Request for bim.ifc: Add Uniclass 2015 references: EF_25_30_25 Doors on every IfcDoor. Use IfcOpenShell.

First a look at what the model holds.

```python
import ifcopenshell

model = ifcopenshell.open("bim.ifc")
print(model.schema)
print("classifications:", [c.Name for c in model.by_type("IfcClassification")])
for ifc_class in ("IfcDoor", "IfcRoof", "IfcStair", "IfcWall", "IfcWindow"):
    print(ifc_class, len(model.by_type(ifc_class)))
```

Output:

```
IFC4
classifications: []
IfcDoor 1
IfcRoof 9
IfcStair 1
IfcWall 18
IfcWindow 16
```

```python
import ifcopenshell
import ifcopenshell.api.classification

model = ifcopenshell.open("bim.ifc")

system = ifcopenshell.api.classification.add_classification(model, classification="Uniclass 2015")

codes = {
    "IfcDoor": ("EF_25_30_25", "Doors"),
}
for ifc_class, (code, name) in codes.items():
    products = model.by_type(ifc_class)
    ifcopenshell.api.classification.add_reference(
        model, products=products, classification=system, identification=code, name=name
    )
    print(code, len(products))

model.write("bim_rev.ifc")
```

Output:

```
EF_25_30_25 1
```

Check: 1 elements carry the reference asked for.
